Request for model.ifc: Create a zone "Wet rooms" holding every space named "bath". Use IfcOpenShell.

First a look at what the model holds.

```python
import ifcopenshell

model = ifcopenshell.open("model.ifc")
print(model.schema)
seen = {}
for space in model.by_type("IfcSpace"):
    seen[space.LongName] = seen.get(space.LongName, 0) + 1
for name, count in sorted(seen.items(), key=str):
    print(count, "x", name)
print("zones:", [z.Name for z in model.by_type("IfcZone")][:20])
```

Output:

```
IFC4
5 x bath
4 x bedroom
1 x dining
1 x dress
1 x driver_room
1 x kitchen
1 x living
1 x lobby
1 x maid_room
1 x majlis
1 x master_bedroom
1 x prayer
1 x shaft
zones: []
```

```python
import ifcopenshell
import ifcopenshell.api.group
import ifcopenshell.api.root

model = ifcopenshell.open("model.ifc")

names = {"bath"}
spaces = [s for s in model.by_type("IfcSpace") if s.LongName in names]

zone = ifcopenshell.api.root.create_entity(model, ifc_class="IfcZone", name="Wet rooms")
ifcopenshell.api.group.assign_group(model, products=spaces, group=zone)
print(len(spaces), "spaces in", zone.Name)

model.write("model_edited.ifc")
```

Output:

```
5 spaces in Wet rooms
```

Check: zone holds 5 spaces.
